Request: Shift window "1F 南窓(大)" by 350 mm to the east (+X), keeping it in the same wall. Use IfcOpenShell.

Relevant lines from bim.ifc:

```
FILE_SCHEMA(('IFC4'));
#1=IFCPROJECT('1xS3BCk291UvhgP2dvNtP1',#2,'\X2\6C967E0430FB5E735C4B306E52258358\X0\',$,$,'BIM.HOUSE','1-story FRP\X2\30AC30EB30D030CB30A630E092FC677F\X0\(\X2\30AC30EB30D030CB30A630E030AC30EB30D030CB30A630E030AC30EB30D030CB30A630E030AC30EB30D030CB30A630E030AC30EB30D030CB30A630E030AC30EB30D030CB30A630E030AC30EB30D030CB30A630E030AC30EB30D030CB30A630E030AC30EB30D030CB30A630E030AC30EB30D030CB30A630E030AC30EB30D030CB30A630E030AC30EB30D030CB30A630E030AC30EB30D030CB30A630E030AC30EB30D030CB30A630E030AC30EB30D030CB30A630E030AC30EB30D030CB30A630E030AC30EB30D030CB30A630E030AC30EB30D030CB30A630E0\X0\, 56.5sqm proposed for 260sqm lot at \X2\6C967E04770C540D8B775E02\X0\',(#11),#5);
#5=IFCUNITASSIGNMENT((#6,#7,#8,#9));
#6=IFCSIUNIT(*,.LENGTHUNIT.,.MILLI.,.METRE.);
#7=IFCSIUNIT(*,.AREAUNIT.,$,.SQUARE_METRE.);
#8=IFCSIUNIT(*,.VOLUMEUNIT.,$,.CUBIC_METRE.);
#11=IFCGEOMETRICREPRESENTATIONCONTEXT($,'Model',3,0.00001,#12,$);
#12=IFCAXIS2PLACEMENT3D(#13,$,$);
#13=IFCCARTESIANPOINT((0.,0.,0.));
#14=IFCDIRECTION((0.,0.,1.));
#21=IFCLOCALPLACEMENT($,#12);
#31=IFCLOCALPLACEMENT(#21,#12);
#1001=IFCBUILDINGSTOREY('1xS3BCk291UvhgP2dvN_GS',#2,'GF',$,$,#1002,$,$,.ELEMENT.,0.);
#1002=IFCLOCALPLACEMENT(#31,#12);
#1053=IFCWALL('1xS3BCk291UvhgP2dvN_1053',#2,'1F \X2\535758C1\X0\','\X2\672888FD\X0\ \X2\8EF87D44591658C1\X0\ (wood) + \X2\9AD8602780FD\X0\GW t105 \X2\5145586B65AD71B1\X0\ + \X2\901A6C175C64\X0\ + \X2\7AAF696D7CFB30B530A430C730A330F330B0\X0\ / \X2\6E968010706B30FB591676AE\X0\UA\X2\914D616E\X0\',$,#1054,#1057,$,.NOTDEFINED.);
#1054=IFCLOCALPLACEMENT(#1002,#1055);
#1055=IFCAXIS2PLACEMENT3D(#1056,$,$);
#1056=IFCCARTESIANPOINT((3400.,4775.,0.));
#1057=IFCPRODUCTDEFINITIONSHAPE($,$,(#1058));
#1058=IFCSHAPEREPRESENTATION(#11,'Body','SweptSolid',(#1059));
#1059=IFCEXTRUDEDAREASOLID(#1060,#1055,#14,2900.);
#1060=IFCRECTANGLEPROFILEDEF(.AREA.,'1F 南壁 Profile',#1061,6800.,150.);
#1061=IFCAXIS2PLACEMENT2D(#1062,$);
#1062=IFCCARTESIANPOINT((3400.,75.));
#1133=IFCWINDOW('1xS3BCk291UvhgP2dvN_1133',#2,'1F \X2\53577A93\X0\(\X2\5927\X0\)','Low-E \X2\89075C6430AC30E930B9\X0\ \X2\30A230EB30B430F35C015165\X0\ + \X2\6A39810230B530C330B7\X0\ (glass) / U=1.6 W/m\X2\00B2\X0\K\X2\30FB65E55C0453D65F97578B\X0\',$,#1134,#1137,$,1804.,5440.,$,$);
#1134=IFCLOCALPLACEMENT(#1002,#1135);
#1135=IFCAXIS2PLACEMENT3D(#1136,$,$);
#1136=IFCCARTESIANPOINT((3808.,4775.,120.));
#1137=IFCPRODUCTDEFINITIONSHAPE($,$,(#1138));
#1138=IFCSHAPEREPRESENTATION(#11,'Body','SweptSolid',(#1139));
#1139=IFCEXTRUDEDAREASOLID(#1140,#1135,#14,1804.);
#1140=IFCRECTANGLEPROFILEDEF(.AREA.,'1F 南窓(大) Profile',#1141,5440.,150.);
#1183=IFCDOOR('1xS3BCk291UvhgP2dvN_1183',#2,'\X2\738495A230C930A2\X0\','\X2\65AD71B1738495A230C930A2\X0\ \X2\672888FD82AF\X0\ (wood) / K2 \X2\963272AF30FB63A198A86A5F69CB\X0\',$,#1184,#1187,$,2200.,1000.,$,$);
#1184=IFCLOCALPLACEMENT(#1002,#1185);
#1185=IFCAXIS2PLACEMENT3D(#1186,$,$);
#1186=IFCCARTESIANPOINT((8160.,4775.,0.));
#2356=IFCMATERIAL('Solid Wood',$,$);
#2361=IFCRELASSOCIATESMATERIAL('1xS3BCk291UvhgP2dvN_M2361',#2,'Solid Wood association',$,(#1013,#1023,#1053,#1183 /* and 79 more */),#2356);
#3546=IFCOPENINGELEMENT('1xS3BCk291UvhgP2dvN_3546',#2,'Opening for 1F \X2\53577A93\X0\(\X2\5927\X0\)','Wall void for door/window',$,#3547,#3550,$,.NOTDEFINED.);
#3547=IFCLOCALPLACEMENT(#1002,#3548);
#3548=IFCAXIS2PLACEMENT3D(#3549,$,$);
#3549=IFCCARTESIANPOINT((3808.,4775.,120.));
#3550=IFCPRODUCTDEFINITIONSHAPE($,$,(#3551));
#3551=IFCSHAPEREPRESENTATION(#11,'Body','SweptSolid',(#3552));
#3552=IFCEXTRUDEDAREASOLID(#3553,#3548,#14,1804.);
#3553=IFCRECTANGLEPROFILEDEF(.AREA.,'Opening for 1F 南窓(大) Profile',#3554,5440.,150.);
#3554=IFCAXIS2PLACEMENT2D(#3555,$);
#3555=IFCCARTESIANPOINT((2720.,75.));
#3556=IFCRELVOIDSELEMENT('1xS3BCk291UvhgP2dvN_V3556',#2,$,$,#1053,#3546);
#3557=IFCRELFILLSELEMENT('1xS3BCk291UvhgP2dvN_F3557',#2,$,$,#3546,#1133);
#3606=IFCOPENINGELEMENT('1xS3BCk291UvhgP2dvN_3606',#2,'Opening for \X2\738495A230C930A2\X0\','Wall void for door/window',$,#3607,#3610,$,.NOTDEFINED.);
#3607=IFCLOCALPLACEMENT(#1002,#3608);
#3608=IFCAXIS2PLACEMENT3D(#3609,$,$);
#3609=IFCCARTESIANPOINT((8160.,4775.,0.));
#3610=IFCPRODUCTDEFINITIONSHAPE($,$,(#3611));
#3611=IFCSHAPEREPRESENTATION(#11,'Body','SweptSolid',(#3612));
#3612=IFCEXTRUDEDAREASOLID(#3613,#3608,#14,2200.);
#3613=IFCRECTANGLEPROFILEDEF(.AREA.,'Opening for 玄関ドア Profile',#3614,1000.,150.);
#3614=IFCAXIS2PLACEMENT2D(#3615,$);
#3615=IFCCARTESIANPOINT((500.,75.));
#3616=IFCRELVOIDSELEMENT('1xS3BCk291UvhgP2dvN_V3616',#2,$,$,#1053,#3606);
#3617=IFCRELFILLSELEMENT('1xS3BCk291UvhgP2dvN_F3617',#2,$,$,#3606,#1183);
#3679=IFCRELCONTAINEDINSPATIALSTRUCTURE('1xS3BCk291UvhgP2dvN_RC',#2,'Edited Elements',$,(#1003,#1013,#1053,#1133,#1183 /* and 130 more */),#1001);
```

```python
import ifcopenshell
import ifcopenshell.api.geometry
import ifcopenshell.util.placement

model = ifcopenshell.open("bim.ifc")

window = model.by_guid("1xS3BCk291UvhgP2dvN_1133")
opening = window.FillsVoids[0].RelatingOpeningElement
wall = opening.VoidsElements[0].RelatingBuildingElement

wall_matrix = ifcopenshell.util.placement.get_local_placement(wall.ObjectPlacement)
shift = wall_matrix[:3, 0] * 350.0
before = ifcopenshell.util.placement.get_local_placement(window.ObjectPlacement)[:3, 3].copy()

# The window is not placed relative to its opening, so move both.
for product in (opening, window):
    matrix = ifcopenshell.util.placement.get_local_placement(product.ObjectPlacement)
    matrix[:3, 3] += shift
    ifcopenshell.api.geometry.edit_object_placement(model, product=product, matrix=matrix, is_si=False)

after = ifcopenshell.util.placement.get_local_placement(window.ObjectPlacement)[:3, 3]
print("window moved by", (after - before).round(3) + 0.0)

model.write("bim_edited.ifc")
```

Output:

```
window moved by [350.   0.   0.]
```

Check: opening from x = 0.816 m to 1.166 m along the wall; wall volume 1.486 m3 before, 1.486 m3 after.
